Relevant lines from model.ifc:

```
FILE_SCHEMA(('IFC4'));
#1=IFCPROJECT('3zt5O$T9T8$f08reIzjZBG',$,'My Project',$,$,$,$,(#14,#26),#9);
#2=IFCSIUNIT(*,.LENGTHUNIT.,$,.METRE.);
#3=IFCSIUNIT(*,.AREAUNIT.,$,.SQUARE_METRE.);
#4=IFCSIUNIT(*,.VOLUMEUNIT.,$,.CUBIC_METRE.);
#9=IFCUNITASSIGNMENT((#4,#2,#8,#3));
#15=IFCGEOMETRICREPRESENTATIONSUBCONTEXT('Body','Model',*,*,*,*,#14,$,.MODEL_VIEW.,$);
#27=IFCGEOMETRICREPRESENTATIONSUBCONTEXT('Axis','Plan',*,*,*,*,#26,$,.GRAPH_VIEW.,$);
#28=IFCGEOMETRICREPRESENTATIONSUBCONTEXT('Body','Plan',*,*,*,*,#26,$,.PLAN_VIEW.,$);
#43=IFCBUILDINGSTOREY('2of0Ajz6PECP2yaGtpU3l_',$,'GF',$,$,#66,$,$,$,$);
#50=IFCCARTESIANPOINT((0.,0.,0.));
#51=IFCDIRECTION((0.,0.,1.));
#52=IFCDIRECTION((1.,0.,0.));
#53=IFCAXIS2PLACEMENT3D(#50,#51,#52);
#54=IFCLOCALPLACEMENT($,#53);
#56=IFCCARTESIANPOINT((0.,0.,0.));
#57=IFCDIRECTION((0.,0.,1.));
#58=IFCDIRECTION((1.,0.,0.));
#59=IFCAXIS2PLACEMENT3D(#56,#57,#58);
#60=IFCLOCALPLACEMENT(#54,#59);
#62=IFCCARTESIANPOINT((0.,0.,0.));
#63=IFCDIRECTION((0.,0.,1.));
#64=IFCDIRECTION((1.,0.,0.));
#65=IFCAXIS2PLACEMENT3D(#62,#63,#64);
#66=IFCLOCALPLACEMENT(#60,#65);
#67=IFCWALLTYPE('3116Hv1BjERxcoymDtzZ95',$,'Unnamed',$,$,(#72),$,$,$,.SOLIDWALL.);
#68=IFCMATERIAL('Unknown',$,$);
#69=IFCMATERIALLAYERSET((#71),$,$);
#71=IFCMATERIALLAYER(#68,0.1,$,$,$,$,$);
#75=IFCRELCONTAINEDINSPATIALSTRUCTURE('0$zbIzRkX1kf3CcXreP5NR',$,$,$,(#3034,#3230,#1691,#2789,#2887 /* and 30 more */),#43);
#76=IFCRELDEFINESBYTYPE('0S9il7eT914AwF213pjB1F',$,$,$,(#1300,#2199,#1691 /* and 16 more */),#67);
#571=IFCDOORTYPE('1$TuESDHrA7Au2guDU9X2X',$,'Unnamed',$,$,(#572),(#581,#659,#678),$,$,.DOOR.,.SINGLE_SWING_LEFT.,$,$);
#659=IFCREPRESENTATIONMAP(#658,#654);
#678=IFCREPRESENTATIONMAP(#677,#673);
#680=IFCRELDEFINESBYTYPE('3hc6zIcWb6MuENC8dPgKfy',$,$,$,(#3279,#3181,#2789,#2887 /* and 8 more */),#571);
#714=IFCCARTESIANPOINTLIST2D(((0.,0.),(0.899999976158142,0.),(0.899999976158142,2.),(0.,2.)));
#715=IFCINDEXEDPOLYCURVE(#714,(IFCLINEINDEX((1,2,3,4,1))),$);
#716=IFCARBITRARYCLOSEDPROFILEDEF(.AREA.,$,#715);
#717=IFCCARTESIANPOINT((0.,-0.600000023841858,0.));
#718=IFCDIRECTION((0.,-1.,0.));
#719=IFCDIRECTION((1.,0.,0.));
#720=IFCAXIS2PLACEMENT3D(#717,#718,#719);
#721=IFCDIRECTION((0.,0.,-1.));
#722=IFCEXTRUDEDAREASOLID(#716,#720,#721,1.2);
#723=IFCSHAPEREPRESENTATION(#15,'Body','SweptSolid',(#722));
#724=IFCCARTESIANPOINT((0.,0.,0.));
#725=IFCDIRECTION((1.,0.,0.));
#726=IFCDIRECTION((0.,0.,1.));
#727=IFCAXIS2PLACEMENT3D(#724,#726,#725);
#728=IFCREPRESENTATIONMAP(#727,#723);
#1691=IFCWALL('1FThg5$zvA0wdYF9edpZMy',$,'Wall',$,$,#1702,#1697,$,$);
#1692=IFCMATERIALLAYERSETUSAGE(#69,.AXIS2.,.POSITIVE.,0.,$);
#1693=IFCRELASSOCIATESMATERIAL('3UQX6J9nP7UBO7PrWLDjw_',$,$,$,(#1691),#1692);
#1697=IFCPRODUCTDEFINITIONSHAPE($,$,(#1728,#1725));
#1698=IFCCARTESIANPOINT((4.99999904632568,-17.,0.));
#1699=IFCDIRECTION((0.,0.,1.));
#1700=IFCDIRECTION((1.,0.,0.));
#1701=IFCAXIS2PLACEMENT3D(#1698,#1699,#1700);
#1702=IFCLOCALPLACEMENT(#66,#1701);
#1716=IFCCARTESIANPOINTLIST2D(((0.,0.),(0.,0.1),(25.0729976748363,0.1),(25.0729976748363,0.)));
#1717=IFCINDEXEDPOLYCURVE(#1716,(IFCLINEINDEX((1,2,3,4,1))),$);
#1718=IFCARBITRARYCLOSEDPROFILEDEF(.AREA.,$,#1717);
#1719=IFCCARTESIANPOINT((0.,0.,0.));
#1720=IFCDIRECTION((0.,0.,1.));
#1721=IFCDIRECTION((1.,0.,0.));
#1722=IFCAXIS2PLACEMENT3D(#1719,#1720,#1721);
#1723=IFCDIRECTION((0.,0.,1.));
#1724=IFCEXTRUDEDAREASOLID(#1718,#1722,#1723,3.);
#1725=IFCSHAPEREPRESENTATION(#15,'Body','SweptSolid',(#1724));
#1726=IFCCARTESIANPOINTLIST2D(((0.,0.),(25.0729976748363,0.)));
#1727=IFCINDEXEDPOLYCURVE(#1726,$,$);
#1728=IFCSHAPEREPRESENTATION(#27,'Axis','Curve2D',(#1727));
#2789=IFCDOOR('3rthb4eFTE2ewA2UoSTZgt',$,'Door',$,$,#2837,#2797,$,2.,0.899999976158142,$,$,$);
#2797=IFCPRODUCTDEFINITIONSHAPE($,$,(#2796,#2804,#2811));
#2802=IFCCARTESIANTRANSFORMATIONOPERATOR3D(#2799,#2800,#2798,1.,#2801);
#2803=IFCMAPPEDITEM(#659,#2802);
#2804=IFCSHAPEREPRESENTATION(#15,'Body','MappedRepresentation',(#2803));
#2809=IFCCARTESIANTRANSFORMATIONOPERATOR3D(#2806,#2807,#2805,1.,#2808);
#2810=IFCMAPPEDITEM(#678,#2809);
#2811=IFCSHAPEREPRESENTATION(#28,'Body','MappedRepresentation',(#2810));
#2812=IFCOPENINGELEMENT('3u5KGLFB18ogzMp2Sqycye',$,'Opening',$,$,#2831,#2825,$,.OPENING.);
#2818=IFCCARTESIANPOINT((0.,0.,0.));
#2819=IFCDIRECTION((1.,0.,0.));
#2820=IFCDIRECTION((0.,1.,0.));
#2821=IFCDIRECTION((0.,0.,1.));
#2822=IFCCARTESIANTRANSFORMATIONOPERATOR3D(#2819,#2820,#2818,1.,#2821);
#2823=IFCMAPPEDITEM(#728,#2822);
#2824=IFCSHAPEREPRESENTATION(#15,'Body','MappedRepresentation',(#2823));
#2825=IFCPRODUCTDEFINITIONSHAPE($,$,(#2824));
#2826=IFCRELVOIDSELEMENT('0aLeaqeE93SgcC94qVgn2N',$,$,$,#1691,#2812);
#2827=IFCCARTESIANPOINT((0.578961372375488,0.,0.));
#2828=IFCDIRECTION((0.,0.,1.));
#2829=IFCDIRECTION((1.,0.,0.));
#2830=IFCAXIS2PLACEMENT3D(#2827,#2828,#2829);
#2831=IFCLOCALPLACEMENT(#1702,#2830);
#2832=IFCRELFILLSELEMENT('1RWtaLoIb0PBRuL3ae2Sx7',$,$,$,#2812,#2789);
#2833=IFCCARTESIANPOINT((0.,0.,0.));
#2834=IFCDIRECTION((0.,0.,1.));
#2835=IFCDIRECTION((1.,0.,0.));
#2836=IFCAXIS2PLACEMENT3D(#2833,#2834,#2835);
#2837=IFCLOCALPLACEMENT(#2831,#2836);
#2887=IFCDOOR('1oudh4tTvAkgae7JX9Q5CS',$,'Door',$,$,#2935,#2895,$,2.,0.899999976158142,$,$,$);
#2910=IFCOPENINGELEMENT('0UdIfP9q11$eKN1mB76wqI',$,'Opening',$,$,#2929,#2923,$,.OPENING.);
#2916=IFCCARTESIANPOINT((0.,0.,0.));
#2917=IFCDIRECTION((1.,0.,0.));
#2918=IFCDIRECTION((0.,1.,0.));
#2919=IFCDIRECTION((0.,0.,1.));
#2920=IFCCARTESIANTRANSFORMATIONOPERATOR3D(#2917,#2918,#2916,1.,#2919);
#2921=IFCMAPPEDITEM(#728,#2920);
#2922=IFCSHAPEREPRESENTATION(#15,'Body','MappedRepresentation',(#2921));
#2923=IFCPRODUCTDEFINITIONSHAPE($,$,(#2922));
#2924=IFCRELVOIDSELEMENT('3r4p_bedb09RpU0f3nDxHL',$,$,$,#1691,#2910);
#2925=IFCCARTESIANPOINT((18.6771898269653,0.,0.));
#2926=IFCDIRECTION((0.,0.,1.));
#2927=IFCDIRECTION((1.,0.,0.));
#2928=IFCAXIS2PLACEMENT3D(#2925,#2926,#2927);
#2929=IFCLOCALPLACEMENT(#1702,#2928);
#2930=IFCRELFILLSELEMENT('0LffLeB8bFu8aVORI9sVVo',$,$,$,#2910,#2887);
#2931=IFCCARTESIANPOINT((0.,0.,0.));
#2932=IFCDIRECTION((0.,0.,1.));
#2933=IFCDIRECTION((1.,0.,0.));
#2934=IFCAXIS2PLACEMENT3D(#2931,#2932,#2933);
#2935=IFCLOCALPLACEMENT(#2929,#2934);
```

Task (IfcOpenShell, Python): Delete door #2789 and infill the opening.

```python
import ifcopenshell
import ifcopenshell.api.feature
import ifcopenshell.api.root
import ifcopenshell.geom
import ifcopenshell.util.shape

model = ifcopenshell.open("model.ifc")
settings = ifcopenshell.geom.settings()


def volume(element):
    """Net volume in cubic metres, openings subtracted."""
    shape = ifcopenshell.geom.create_shape(settings, element)
    return ifcopenshell.util.shape.get_volume(shape.geometry)


door = model.by_guid("3rthb4eFTE2ewA2UoSTZgt")
opening = door.FillsVoids[0].RelatingOpeningElement
wall = opening.VoidsElements[0].RelatingBuildingElement
before = volume(wall)

ifcopenshell.api.root.remove_product(model, product=door)
ifcopenshell.api.feature.remove_feature(model, feature=opening)

after = volume(wall)

print(f"wall volume {before:.3f} -> {after:.3f} m3")

model.write("model_v2.ifc")
```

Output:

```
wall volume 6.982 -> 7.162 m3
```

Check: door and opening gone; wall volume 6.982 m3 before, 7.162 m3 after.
